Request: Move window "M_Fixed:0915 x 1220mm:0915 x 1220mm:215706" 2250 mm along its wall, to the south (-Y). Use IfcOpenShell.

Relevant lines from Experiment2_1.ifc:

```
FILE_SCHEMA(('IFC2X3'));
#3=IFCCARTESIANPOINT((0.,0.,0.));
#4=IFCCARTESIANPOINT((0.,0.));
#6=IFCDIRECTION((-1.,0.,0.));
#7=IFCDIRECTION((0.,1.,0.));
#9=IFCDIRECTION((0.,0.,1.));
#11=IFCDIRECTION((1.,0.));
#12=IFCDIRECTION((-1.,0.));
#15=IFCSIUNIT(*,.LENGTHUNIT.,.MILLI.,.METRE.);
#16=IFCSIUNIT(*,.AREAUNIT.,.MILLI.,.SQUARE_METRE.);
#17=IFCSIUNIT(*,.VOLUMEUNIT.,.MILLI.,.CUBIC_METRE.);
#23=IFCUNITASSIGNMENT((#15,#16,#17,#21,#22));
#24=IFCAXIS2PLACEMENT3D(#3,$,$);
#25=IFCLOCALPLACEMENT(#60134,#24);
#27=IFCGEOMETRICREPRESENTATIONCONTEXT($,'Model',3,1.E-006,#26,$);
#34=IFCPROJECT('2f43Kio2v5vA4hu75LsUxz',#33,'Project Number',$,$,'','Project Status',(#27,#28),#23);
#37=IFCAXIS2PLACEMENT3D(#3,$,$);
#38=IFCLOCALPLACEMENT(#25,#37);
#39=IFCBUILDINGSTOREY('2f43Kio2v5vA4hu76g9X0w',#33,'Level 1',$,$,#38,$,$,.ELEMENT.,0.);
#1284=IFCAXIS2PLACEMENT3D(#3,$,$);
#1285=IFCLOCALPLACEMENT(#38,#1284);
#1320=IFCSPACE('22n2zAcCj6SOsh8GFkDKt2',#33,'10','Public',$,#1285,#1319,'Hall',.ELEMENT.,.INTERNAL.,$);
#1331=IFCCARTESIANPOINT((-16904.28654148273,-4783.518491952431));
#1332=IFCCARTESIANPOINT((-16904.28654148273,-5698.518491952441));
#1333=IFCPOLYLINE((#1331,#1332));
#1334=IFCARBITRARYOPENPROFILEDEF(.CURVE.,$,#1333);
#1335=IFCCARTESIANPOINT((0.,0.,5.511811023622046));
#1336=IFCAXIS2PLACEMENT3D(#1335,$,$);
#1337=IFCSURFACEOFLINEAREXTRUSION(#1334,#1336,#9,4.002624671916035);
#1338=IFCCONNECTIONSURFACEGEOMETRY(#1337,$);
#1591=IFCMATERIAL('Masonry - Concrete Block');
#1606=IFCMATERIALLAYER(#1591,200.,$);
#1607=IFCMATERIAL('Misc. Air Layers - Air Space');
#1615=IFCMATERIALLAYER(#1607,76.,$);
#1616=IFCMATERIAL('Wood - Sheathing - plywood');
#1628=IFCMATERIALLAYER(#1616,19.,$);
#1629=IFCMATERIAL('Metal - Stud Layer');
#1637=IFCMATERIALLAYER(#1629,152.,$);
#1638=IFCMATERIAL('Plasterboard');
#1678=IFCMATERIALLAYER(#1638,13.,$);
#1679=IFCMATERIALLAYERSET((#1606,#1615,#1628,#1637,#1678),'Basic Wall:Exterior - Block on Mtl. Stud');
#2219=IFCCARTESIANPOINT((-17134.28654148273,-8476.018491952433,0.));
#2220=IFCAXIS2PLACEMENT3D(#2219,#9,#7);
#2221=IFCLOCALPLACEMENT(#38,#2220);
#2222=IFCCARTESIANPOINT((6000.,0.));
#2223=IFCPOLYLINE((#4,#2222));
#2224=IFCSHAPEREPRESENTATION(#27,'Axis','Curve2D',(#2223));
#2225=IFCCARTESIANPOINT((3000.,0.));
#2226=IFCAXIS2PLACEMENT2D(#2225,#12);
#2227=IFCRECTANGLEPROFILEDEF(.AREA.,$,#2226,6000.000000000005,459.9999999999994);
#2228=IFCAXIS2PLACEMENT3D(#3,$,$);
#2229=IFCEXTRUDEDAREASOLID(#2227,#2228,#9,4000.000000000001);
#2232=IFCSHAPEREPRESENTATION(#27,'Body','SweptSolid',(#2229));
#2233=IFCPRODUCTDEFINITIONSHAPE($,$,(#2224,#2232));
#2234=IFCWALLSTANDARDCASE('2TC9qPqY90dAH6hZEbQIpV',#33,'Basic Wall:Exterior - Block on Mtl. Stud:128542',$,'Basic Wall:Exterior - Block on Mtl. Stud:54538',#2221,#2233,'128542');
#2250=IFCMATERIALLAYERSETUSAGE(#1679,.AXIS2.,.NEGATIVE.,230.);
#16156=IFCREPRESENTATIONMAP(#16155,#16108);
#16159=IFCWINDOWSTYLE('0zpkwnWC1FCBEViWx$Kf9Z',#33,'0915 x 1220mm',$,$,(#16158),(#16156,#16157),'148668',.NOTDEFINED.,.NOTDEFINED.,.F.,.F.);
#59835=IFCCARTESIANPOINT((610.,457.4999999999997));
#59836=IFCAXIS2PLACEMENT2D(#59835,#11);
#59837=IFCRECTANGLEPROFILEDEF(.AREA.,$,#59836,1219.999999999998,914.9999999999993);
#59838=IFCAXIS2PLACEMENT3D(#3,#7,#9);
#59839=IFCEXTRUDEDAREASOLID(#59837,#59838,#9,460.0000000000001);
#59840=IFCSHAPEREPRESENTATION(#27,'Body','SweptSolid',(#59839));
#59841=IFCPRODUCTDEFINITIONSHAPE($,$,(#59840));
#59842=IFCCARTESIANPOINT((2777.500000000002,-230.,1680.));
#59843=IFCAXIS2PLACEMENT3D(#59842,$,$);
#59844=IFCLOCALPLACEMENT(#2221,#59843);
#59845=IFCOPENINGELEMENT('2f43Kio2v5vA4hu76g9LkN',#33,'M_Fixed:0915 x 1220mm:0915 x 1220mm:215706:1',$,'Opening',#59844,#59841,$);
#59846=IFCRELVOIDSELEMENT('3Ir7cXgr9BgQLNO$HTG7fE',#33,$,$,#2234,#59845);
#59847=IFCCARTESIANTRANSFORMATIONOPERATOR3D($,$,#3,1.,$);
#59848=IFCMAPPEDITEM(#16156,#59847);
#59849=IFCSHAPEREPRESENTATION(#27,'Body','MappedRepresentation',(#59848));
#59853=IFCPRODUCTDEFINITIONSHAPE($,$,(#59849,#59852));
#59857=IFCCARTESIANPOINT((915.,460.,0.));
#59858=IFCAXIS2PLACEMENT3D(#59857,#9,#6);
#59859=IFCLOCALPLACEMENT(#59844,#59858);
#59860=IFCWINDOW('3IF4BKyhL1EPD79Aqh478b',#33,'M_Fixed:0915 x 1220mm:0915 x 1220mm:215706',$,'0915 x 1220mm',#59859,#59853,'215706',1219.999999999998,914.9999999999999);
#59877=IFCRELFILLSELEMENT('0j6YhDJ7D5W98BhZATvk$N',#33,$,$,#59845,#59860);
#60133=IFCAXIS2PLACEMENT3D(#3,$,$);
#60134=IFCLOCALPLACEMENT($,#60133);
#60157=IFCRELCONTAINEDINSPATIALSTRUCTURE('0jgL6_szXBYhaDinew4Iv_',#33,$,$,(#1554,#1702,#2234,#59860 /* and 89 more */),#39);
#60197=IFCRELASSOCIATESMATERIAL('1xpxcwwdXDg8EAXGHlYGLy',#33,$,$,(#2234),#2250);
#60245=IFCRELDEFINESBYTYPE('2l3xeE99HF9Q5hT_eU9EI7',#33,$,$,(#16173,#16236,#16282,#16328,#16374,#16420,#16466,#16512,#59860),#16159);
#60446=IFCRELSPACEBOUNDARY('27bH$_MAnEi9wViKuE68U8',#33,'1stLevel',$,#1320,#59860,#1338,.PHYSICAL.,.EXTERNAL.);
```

```python
import numpy as np
import ifcopenshell
import ifcopenshell.api.geometry
import ifcopenshell.util.placement
import ifcopenshell.util.unit

model = ifcopenshell.open("Experiment2_1.ifc")
unit_scale = ifcopenshell.util.unit.calculate_unit_scale(model)

window = model.by_id(59860)
opening = window.FillsVoids[0].RelatingOpeningElement
wall = opening.VoidsElements[0].RelatingBuildingElement

wall_matrix = ifcopenshell.util.placement.get_local_placement(wall.ObjectPlacement)
shift = wall_matrix[:3, 0] * -2.25 / unit_scale
before = ifcopenshell.util.placement.get_local_placement(window.ObjectPlacement)[:3, 3].copy()

# The window is placed relative to its opening, so it follows when the opening moves.
matrix = ifcopenshell.util.placement.get_local_placement(opening.ObjectPlacement)
matrix[:3, 3] += shift
ifcopenshell.api.geometry.edit_object_placement(
    model, product=opening, matrix=matrix, is_si=False, should_transform_children=True
)

# Space boundary surfaces are stored in each space's coordinates; move them too.
for rel in window.ProvidesBoundaries:
    if not rel.ConnectionGeometry:
        continue
    surface = rel.ConnectionGeometry.SurfaceOnRelatingElement
    space_matrix = ifcopenshell.util.placement.get_local_placement(rel.RelatingSpace.ObjectPlacement)
    point = np.array(surface.Position.Location.Coordinates) + space_matrix[:3, :3].T @ shift
    surface.Position = model.createIfcAxis2Placement3D(
        model.createIfcCartesianPoint(point.tolist()), surface.Position.Axis, surface.Position.RefDirection
    )

after = ifcopenshell.util.placement.get_local_placement(window.ObjectPlacement)[:3, 3]
print("window moved by", (after - before).round(3) + 0.0)

model.write("Experiment2_1_edited.ifc")
```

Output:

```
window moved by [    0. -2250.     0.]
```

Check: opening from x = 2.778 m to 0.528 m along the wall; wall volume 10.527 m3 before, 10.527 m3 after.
